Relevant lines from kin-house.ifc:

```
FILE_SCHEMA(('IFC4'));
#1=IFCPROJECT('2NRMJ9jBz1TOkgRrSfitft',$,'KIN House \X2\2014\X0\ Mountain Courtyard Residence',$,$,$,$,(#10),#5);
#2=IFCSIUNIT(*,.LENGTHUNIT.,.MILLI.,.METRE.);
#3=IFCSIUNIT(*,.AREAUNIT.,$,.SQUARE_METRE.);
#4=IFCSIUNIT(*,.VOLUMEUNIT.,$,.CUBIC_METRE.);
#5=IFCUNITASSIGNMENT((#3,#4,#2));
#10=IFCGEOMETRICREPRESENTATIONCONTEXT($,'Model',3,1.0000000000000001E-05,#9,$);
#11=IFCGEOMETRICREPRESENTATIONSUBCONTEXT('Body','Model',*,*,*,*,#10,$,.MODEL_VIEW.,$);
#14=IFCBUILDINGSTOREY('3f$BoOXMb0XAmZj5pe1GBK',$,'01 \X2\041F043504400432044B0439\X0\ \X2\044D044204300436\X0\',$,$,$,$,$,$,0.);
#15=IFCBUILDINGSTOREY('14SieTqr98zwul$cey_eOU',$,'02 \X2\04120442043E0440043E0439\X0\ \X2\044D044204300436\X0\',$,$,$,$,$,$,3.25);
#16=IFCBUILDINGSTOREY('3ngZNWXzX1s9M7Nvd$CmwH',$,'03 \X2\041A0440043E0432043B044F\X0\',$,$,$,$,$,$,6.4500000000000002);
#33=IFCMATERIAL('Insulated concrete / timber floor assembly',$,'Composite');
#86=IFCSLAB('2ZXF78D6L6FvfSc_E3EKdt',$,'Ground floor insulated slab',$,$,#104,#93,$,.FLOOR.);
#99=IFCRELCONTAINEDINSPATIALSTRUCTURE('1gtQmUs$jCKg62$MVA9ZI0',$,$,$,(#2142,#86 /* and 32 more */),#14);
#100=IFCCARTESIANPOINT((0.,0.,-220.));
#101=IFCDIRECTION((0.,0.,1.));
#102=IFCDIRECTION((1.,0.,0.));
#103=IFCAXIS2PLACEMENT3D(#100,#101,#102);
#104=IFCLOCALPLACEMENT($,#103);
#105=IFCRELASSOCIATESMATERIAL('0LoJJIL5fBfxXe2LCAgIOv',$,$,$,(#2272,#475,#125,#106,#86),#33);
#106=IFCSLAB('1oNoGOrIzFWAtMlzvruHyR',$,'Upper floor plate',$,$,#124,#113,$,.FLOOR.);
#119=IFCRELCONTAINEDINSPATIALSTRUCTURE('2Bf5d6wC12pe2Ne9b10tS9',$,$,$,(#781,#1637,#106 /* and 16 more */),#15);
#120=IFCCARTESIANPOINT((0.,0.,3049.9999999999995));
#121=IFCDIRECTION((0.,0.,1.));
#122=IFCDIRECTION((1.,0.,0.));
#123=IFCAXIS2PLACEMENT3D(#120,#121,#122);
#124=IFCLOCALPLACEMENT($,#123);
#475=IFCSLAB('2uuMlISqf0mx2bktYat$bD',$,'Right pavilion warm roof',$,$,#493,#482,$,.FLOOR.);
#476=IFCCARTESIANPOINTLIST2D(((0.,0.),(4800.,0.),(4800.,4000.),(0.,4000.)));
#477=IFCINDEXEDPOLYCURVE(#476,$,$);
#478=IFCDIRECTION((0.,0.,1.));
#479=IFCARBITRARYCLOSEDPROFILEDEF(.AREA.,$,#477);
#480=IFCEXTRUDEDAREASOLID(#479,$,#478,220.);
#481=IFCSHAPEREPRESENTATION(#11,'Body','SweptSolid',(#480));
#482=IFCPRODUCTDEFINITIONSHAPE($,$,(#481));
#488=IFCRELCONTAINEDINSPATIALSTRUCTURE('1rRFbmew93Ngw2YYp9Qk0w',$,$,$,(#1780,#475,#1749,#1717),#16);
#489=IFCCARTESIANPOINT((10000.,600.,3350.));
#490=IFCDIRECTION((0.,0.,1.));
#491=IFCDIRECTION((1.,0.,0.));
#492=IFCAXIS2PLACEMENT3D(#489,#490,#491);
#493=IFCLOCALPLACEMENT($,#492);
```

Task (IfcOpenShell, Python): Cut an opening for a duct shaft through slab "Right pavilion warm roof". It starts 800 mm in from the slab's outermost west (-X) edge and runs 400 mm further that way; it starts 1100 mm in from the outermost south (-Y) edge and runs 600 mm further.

```python
import numpy as np
import ifcopenshell
import ifcopenshell.api.feature
import ifcopenshell.api.geometry
import ifcopenshell.api.root
import ifcopenshell.geom
import ifcopenshell.util.placement
import ifcopenshell.util.representation
import ifcopenshell.util.shape
import ifcopenshell.util.unit

model = ifcopenshell.open("kin-house.ifc")
unit_scale = ifcopenshell.util.unit.calculate_unit_scale(model)
settings = ifcopenshell.geom.settings()


def volume(element):
    """Net volume in cubic metres, openings subtracted."""
    shape = ifcopenshell.geom.create_shape(settings, element)
    return ifcopenshell.util.shape.get_volume(shape.geometry)


slab = model.by_id(475)
before = volume(slab)

# Extent in the slab's own axes, in metres. The edges named are its -X and -Y sides.
slab_shape = ifcopenshell.geom.create_shape(settings, slab)
vertices = ifcopenshell.util.shape.get_vertices(slab_shape.geometry)
x_min, y_min, bottom = vertices.min(axis=0)
top = vertices[:, 2].max()

opening = ifcopenshell.api.root.create_entity(model, ifc_class="IfcOpeningElement", name="Duct shaft opening", predefined_type="OPENING")
context = ifcopenshell.util.representation.get_context(model, "Model", "Body", "MODEL_VIEW")
width, depth = 0.4, 0.6
outline = [(0.0, 0.0), (width, 0.0), (width, depth), (0.0, depth), (0.0, 0.0)]
# Overshoot both faces by 50 mm so the cut is clean.
shape = ifcopenshell.api.geometry.add_slab_representation(
    model, context=context, depth=top - bottom + 0.1, polyline=outline
)
ifcopenshell.api.geometry.assign_representation(model, product=opening, representation=shape)

matrix = ifcopenshell.util.placement.get_local_placement(slab.ObjectPlacement)
matrix[:, 3] = matrix @ np.append(np.array([x_min + 0.8, y_min + 1.1, bottom - 0.05]) / unit_scale, 1.0)
ifcopenshell.api.geometry.edit_object_placement(model, product=opening, matrix=matrix, is_si=False)
ifcopenshell.api.feature.add_feature(model, feature=opening, element=slab)

after = volume(slab)

print(f"slab volume {before:.3f} -> {after:.3f} m3")

model.write("kin-house_v2.ifc")
```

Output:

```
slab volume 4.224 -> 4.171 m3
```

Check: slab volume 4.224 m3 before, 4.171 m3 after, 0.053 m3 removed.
